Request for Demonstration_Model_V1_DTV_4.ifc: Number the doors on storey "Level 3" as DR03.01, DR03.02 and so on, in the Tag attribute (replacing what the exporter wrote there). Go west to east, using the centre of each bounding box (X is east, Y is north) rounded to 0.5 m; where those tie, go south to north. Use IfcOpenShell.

First a look at what the model holds.

```python
import ifcopenshell
import ifcopenshell.util.element
import ifcopenshell.util.placement

model = ifcopenshell.open("Demonstration_Model_V1_DTV_4.ifc")
print(model.schema)
storey = next(s for s in model.by_type("IfcBuildingStorey") if s.Name == "Level 3")
doors = [e for e in ifcopenshell.util.element.get_decomposition(storey) if e.is_a("IfcDoor")]
for e in sorted(doors, key=lambda e: e.id()):
    origin = ifcopenshell.util.placement.get_local_placement(e.ObjectPlacement)[:3, 3]
    print(e.id(), e.Tag, e.Name, origin.round(2) + 0.0, sep=" | ")
```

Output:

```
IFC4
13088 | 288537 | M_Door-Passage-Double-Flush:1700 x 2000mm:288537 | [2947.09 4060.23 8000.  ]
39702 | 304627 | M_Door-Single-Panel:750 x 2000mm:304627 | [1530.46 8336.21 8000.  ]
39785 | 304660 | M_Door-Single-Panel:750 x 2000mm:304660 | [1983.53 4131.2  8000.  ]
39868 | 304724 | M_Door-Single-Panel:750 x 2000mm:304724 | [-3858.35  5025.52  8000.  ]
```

```python
import ifcopenshell
import ifcopenshell.geom
import ifcopenshell.util.element
import ifcopenshell.util.shape

model = ifcopenshell.open("Demonstration_Model_V1_DTV_4.ifc")
settings = ifcopenshell.geom.settings()
settings.set("use-world-coords", True)


def centre(element):
    shape = ifcopenshell.geom.create_shape(settings, element)
    return ifcopenshell.util.shape.get_bbox_centroid(shape.geometry)


storey = next(s for s in model.by_type("IfcBuildingStorey") if s.Name == "Level 3")
doors = [e for e in ifcopenshell.util.element.get_decomposition(storey) if e.is_a("IfcDoor")]

# Insertion points can sit at a corner or the storey origin, so sort by the geometry (in metres).
centres = {e: centre(e) for e in doors}
doors.sort(key=lambda e: (round(centres[e][0] / 0.5), centres[e][1]))

for i, e in enumerate(doors, start=1):
    number = f"DR03.{i:02d}"
    e.Tag = number
    print(e.id(), number)

model.write("Demonstration_Model_V1_DTV_4_rev.ifc")
```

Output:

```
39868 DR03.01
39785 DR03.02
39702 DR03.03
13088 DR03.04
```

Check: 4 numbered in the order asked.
